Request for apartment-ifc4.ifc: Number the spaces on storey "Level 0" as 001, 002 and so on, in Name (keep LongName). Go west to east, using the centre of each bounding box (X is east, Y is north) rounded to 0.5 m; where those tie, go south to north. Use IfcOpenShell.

First a look at what the model holds.

```python
import ifcopenshell
import ifcopenshell.util.element
import ifcopenshell.util.placement

model = ifcopenshell.open("apartment-ifc4.ifc")
print(model.schema)
storey = next(s for s in model.by_type("IfcBuildingStorey") if s.Name == "Level 0")
spaces = [e for e in ifcopenshell.util.element.get_decomposition(storey) if e.is_a("IfcSpace")]
for e in sorted(spaces, key=lambda e: e.id()):
    origin = ifcopenshell.util.placement.get_local_placement(e.ObjectPlacement)[:3, 3]
    print(e.id(), e.Name, e.LongName, origin.round(2) + 0.0, sep=" | ")
```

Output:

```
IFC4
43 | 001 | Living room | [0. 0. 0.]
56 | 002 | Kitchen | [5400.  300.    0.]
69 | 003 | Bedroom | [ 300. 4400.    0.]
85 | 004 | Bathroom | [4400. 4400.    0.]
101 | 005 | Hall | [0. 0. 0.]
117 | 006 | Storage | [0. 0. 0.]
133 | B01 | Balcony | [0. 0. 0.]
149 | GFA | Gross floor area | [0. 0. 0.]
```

```python
import ifcopenshell
import ifcopenshell.geom
import ifcopenshell.util.element
import ifcopenshell.util.shape

model = ifcopenshell.open("apartment-ifc4.ifc")
settings = ifcopenshell.geom.settings()
settings.set("use-world-coords", True)


def centre(element):
    shape = ifcopenshell.geom.create_shape(settings, element)
    return ifcopenshell.util.shape.get_bbox_centroid(shape.geometry)


storey = next(s for s in model.by_type("IfcBuildingStorey") if s.Name == "Level 0")
spaces = [e for e in ifcopenshell.util.element.get_decomposition(storey) if e.is_a("IfcSpace")]

# Insertion points can sit at a corner or the storey origin, so sort by the geometry (in metres).
centres = {e: centre(e) for e in spaces}
spaces.sort(key=lambda e: (round(centres[e][0] / 0.5), centres[e][1]))

for i, e in enumerate(spaces, start=1):
    number = f"0{i:02d}"
    e.Name = number
    print(e.id(), number)

model.write("apartment-ifc4_v2.ifc")
```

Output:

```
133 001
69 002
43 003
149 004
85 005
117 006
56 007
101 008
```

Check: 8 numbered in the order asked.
